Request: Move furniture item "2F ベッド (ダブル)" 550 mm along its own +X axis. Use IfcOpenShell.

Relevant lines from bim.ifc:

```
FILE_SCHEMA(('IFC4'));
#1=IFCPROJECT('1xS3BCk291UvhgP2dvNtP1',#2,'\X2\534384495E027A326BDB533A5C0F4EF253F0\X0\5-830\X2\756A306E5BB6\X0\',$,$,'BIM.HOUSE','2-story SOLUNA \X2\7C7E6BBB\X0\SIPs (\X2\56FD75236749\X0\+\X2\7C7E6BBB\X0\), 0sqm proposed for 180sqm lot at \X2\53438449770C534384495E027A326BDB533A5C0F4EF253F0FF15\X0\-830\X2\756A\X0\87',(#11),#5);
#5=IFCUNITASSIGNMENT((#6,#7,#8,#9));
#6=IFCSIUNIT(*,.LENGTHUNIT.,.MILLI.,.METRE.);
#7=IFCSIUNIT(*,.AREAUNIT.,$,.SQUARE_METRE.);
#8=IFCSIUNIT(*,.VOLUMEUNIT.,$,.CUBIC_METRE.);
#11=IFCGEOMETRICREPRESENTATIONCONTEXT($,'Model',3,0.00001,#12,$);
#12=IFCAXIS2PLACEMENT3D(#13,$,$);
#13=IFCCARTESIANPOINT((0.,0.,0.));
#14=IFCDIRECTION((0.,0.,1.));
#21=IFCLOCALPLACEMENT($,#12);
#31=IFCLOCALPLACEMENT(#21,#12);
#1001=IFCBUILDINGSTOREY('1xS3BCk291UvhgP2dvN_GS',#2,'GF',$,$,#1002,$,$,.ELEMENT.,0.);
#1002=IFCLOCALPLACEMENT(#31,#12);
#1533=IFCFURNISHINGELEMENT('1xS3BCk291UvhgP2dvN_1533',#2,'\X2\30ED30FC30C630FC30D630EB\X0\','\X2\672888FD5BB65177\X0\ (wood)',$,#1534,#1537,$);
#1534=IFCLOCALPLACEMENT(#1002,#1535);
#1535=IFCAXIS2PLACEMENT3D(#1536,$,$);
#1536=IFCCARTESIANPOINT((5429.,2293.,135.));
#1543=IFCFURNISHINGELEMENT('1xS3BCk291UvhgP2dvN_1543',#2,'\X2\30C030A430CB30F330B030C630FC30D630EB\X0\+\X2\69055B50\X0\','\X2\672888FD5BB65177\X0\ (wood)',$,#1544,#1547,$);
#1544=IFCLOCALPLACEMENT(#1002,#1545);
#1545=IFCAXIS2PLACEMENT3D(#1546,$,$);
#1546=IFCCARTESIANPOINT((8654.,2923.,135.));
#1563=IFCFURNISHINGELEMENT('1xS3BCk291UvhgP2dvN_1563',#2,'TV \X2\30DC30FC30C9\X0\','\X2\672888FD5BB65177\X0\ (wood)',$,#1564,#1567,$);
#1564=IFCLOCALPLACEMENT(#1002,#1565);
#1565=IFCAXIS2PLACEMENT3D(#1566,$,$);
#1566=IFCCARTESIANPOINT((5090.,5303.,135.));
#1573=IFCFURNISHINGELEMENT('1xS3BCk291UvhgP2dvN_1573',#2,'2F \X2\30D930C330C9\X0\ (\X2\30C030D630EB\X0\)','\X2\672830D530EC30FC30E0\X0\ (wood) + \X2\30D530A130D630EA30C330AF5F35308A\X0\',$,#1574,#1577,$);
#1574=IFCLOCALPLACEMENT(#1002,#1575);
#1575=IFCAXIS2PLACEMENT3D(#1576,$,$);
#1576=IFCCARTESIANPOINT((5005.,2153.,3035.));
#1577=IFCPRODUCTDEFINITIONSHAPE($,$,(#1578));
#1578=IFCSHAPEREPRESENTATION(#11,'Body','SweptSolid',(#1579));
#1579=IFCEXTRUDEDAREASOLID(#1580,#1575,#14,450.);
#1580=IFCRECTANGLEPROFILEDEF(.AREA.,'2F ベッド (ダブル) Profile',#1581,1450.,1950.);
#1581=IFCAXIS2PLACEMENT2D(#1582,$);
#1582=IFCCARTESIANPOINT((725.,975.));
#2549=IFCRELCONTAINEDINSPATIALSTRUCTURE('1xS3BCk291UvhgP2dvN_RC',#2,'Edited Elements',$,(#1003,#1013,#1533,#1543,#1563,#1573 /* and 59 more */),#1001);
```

```python
import ifcopenshell
import ifcopenshell.api.geometry
import ifcopenshell.util.placement
import ifcopenshell.util.unit

model = ifcopenshell.open("bim.ifc")
unit_scale = ifcopenshell.util.unit.calculate_unit_scale(model)

item = model.by_id(1573)
matrix = ifcopenshell.util.placement.get_local_placement(item.ObjectPlacement)
matrix[:3, 3] += matrix[:3, 0] * 0.55 / unit_scale
ifcopenshell.api.geometry.edit_object_placement(model, product=item, matrix=matrix, is_si=False)

print(ifcopenshell.util.placement.get_local_placement(item.ObjectPlacement).round(3) + 0.0)

model.write("bim_v2.ifc")
```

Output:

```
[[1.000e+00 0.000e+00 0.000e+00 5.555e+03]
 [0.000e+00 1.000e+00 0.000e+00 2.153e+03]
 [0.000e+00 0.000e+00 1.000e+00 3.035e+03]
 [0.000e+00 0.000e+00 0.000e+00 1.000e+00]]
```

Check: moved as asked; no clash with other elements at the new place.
